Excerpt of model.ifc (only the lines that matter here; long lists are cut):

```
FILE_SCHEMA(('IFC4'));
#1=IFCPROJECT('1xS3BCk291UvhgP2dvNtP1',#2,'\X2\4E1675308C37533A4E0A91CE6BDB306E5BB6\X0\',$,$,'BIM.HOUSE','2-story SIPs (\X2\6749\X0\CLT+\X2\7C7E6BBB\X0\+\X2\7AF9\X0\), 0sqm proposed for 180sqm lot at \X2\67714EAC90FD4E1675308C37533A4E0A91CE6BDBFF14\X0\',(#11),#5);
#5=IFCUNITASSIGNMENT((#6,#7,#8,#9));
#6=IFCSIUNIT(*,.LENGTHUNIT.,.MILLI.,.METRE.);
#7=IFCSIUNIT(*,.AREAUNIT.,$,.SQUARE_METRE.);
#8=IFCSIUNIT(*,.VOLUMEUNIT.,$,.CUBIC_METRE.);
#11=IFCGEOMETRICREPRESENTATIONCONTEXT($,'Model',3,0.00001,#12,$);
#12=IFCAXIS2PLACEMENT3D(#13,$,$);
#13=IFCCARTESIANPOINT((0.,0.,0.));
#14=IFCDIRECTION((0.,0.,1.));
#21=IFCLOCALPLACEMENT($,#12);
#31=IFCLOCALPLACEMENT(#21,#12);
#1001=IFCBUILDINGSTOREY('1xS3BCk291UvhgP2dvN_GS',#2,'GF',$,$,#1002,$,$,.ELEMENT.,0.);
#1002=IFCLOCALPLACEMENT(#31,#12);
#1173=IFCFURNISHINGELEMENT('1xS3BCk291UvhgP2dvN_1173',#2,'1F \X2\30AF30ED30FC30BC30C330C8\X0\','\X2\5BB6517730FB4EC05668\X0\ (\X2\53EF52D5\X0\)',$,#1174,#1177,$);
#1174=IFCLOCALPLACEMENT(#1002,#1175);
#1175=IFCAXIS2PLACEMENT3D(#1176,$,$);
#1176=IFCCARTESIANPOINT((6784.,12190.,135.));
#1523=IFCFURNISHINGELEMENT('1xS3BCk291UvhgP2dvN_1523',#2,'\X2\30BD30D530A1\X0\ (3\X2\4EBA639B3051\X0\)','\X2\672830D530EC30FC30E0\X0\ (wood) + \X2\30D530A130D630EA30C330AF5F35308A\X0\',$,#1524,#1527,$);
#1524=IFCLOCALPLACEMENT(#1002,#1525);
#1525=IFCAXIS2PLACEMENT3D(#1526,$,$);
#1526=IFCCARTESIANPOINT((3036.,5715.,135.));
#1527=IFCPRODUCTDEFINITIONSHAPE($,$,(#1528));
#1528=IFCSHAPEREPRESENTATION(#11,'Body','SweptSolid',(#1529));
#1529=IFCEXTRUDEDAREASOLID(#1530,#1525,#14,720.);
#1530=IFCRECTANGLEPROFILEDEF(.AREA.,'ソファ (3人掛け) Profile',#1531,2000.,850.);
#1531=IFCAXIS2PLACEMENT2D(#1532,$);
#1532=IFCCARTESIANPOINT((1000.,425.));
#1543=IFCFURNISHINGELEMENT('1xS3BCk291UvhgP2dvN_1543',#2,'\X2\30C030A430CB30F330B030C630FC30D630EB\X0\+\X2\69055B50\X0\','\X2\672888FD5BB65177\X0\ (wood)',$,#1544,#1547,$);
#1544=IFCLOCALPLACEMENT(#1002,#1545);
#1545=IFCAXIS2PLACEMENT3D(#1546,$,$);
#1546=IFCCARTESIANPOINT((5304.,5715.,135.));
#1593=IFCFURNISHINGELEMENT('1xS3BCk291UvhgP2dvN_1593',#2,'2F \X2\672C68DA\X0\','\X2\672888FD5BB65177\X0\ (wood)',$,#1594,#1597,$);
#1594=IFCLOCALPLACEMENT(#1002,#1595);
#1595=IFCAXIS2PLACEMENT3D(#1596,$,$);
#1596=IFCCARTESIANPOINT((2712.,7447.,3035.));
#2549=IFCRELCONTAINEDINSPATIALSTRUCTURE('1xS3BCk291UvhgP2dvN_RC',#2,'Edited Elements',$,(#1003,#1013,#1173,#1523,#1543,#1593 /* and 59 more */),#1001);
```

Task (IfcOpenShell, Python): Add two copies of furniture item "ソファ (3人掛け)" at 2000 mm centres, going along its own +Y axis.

```python
import ifcopenshell
import ifcopenshell.api.geometry
import ifcopenshell.api.root
import ifcopenshell.util.element
import ifcopenshell.util.placement

model = ifcopenshell.open("model.ifc")


def reuse_history(source, copy):
    """copy_class also copies each property set's owner history, people and application; keep the originals."""
    for rel in copy.IsDefinedBy:
        if rel.is_a("IfcRelDefinesByProperties") and (history := rel.RelatingPropertyDefinition.OwnerHistory):
            rel.RelatingPropertyDefinition.OwnerHistory = source.OwnerHistory
            ifcopenshell.util.element.remove_deep2(model, history)


source = model.by_guid("1xS3BCk291UvhgP2dvN_1523")
base = ifcopenshell.util.placement.get_local_placement(source.ObjectPlacement)
step = base[:3, 1] * 2000.0

for i in range(1, 3):
    copy = ifcopenshell.api.root.copy_class(model, product=source)
    copy.Representation = ifcopenshell.util.element.copy_deep(
        model, source.Representation, exclude=["IfcGeometricRepresentationContext", "IfcRepresentationMap"]
    )
    reuse_history(source, copy)
    matrix = base.copy()
    matrix[:3, 3] += i * step
    print("added at", matrix[:3, 3].round(3) + 0.0)
    ifcopenshell.api.geometry.edit_object_placement(model, product=copy, matrix=matrix, is_si=False)

model.write("model_rev.ifc")
```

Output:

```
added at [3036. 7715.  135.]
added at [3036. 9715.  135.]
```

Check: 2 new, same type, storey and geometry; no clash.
